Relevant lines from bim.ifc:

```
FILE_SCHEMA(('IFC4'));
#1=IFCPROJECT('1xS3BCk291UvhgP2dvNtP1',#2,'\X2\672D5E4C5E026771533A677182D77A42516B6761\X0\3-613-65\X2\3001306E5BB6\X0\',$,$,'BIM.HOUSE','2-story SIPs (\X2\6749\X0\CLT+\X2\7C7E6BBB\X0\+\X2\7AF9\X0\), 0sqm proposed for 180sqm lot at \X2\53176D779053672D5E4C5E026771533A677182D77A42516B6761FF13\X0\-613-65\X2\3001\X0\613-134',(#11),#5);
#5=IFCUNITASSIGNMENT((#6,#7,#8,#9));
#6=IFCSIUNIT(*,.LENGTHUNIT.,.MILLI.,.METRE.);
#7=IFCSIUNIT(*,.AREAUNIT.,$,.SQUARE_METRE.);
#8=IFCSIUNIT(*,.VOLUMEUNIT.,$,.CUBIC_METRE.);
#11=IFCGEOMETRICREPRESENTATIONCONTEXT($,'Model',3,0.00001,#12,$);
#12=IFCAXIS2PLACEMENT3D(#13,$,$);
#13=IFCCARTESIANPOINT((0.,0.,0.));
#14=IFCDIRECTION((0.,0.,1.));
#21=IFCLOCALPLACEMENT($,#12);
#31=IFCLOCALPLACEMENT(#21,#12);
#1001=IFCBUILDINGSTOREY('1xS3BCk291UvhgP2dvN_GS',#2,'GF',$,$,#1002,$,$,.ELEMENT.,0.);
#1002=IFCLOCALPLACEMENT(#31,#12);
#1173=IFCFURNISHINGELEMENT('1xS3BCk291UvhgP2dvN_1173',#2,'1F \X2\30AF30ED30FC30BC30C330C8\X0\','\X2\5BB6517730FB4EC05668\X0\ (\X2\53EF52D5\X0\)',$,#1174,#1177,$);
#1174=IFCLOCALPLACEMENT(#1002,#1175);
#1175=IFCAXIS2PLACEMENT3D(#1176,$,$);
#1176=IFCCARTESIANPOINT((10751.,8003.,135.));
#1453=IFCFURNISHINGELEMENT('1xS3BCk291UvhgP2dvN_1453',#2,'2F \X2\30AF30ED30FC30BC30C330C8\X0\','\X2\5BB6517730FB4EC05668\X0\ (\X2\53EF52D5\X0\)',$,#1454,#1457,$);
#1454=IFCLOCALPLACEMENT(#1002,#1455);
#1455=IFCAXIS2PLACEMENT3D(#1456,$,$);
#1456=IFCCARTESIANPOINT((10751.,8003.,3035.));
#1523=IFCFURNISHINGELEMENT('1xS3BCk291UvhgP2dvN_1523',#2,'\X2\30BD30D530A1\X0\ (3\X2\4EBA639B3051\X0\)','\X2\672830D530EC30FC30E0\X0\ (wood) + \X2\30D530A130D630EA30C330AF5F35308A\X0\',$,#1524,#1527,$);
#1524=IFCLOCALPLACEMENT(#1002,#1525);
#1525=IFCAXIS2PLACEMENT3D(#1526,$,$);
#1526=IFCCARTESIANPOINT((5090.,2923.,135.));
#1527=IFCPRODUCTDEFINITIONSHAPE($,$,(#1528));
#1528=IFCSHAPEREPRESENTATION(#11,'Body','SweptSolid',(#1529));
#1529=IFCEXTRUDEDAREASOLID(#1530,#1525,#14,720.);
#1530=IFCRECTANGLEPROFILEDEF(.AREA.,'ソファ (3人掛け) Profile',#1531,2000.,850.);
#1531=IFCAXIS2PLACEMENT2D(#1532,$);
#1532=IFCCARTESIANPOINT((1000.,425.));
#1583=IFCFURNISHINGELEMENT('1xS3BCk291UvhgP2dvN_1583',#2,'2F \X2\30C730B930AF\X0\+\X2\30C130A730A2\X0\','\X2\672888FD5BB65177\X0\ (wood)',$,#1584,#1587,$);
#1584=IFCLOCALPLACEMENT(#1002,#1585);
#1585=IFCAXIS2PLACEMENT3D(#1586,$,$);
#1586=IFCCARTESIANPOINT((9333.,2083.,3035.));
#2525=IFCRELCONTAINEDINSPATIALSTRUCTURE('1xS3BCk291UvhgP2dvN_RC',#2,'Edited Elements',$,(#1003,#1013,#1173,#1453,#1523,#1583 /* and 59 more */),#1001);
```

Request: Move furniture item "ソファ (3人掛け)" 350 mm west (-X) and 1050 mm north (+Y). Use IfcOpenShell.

```python
import ifcopenshell
import ifcopenshell.api.geometry
import ifcopenshell.util.placement

model = ifcopenshell.open("bim.ifc")

item = model.by_guid("1xS3BCk291UvhgP2dvN_1523")
matrix = ifcopenshell.util.placement.get_local_placement(item.ObjectPlacement)
matrix[0, 3] -= 350.0
matrix[1, 3] += 1050.0
ifcopenshell.api.geometry.edit_object_placement(model, product=item, matrix=matrix, is_si=False)

print(ifcopenshell.util.placement.get_local_placement(item.ObjectPlacement).round(3) + 0.0)

model.write("bim-out.ifc")
```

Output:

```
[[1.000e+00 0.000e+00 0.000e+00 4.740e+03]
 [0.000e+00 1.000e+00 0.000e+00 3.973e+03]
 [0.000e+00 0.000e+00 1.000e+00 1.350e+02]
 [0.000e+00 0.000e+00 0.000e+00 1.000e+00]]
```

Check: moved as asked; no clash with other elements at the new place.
